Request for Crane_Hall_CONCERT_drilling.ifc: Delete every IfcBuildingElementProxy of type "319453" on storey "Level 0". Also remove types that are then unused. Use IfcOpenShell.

First a look at what the model holds.

```python
import ifcopenshell
import ifcopenshell.util.element

model = ifcopenshell.open("Crane_Hall_CONCERT_drilling.ifc")
print(model.schema)
storey = next(s for s in model.by_type("IfcBuildingStorey") if s.Name == "Level 0")
proxies = [e for e in ifcopenshell.util.element.get_decomposition(storey) if e.is_a("IfcBuildingElementProxy")]
seen = {}
for e in proxies:
    element_type = ifcopenshell.util.element.get_type(e)
    name = element_type.Name if element_type not in (None, e) else None
    seen[name] = seen.get(name, 0) + 1
for name, count in sorted(seen.items(), key=str):
    print(count, "x", name)
```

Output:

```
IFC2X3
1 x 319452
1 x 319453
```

```python
import ifcopenshell
import ifcopenshell.api.root
import ifcopenshell.util.element

model = ifcopenshell.open("Crane_Hall_CONCERT_drilling.ifc")

storey = next(s for s in model.by_type("IfcBuildingStorey") if s.Name == "Level 0")
proxies = [e for e in ifcopenshell.util.element.get_decomposition(storey) if e.is_a("IfcBuildingElementProxy")]
targets = [e for e in proxies if (t := ifcopenshell.util.element.get_type(e)) not in (None, e) and t.Name == "319453"]
types = {ifcopenshell.util.element.get_type(e) for e in targets} - {None, *targets}

for e in targets:
    ifcopenshell.api.root.remove_product(model, product=e)
print(len(targets), "removed")

unused = [t for t in types if not ifcopenshell.util.element.get_types(t)]
for t in unused:
    ifcopenshell.api.root.remove_product(model, product=t)
print(len(unused), "unused types removed")

model.write("Crane_Hall_CONCERT_drilling_rev.ifc")
```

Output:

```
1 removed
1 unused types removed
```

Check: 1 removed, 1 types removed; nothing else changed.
